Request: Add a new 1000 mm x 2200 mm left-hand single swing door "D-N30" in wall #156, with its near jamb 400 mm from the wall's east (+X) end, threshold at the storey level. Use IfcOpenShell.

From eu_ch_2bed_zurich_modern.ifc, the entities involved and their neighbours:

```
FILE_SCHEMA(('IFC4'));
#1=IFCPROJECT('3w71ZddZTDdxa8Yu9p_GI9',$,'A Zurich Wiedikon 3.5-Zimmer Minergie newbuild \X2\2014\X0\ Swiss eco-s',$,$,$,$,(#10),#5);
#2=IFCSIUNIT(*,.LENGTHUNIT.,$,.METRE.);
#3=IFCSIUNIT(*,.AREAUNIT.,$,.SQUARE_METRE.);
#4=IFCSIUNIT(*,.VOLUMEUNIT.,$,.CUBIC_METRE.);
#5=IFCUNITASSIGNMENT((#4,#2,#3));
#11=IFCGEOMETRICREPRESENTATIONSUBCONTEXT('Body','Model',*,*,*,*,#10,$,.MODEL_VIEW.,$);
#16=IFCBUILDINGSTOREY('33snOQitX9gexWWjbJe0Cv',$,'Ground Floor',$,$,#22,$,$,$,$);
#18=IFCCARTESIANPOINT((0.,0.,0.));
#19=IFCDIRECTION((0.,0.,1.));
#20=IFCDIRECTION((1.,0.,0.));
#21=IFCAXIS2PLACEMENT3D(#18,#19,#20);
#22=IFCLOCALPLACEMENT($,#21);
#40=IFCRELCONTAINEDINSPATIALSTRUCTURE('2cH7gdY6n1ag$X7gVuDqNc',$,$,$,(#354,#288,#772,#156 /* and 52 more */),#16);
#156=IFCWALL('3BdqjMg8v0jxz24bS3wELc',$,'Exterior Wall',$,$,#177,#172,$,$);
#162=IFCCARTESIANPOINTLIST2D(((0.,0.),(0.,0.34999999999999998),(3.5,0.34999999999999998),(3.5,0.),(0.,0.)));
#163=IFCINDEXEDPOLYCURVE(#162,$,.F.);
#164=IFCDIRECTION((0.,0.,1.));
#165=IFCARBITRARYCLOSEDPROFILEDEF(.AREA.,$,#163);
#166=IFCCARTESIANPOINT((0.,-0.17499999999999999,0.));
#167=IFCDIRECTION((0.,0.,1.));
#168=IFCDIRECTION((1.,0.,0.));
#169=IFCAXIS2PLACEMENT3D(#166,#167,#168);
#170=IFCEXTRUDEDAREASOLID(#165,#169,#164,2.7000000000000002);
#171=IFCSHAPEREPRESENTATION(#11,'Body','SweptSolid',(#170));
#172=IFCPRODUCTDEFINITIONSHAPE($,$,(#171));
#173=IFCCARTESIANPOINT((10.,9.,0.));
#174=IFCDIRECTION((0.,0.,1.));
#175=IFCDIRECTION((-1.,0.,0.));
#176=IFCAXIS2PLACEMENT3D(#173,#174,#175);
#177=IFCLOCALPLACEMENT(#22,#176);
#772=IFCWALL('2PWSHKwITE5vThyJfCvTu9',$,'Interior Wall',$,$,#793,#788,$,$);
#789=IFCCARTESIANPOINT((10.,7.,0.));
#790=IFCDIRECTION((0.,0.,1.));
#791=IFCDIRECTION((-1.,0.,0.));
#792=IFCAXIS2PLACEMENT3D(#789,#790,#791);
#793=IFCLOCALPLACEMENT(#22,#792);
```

```python
import numpy as np
import ifcopenshell
import ifcopenshell.api.feature
import ifcopenshell.api.geometry
import ifcopenshell.api.root
import ifcopenshell.api.spatial
import ifcopenshell.geom
import ifcopenshell.util.element
import ifcopenshell.util.placement
import ifcopenshell.util.representation
import ifcopenshell.util.shape
import ifcopenshell.util.unit

model = ifcopenshell.open("eu_ch_2bed_zurich_modern.ifc")
unit_scale = ifcopenshell.util.unit.calculate_unit_scale(model)
settings = ifcopenshell.geom.settings()


def volume(element):
    """Net volume in cubic metres, openings subtracted."""
    shape = ifcopenshell.geom.create_shape(settings, element)
    return ifcopenshell.util.shape.get_volume(shape.geometry)


wall = model.by_guid("3BdqjMg8v0jxz24bS3wELc")
storey = ifcopenshell.util.element.get_container(wall, ifc_class="IfcBuildingStorey")
context = ifcopenshell.util.representation.get_context(model, "Model", "Body", "MODEL_VIEW")
before = volume(wall)

width, height, from_end, sill = 1, 2.2, 0.4, 0.0  # metres

# The wall runs along its own X axis, and the end named is its -X end.
wall_shape = ifcopenshell.geom.create_shape(settings, wall)
x, y, z = ifcopenshell.util.shape.get_vertices(wall_shape.geometry).T
start = x.min() + from_end
face, thickness = float(y.min()), float(y.max() - y.min())
wall_matrix = ifcopenshell.util.placement.get_local_placement(wall.ObjectPlacement)
level = ifcopenshell.util.placement.get_local_placement(storey.ObjectPlacement)[2, 3]


def in_wall(x, y):
    """Placement at x, y metres in the wall's axes, at sill height."""
    matrix = wall_matrix.copy()
    matrix[:, 3] = wall_matrix @ np.array([x / unit_scale, y / unit_scale, 0.0, 1.0])
    matrix[2, 3] = level + sill / unit_scale
    return matrix


# Opening: a box that overshoots both wall faces by 50 mm.
opening = ifcopenshell.api.root.create_entity(model, ifc_class="IfcOpeningElement", predefined_type="OPENING")
box = ifcopenshell.api.geometry.add_wall_representation(
    model, context=context, length=width, height=height, thickness=thickness + 0.1
)
ifcopenshell.api.geometry.assign_representation(model, product=opening, representation=box)
ifcopenshell.api.geometry.edit_object_placement(model, product=opening, matrix=in_wall(start, face - 0.05), is_si=False)
ifcopenshell.api.feature.add_feature(model, feature=opening, element=wall)

door = ifcopenshell.api.root.create_entity(model, ifc_class="IfcDoor", name="D-N30", predefined_type="DOOR")
door.OverallWidth, door.OverallHeight = width / unit_scale, height / unit_scale
door.OperationType = "SINGLE_SWING_LEFT"
body = ifcopenshell.api.geometry.add_door_representation(
    model,
    context=context,
    overall_width=door.OverallWidth,
    overall_height=door.OverallHeight,
    operation_type="SINGLE_SWING_LEFT",
    lining_properties={"LiningDepth": thickness / unit_scale, "ThresholdDepth": thickness / unit_scale},
)
ifcopenshell.api.geometry.assign_representation(model, product=door, representation=body)
ifcopenshell.api.spatial.assign_container(model, products=[door], relating_structure=storey)
ifcopenshell.api.feature.add_filling(model, opening=opening, element=door)

# The lining spans the wall, so the door starts at the wall face.
ifcopenshell.api.geometry.edit_object_placement(model, product=door, matrix=in_wall(start, face), is_si=False)

after = volume(wall)

print(f"wall volume {before:.3f} -> {after:.3f} m3")

model.write("eu_ch_2bed_zurich_modern_v2.ifc")
```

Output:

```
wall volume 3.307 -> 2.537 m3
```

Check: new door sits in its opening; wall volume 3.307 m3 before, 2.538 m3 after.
